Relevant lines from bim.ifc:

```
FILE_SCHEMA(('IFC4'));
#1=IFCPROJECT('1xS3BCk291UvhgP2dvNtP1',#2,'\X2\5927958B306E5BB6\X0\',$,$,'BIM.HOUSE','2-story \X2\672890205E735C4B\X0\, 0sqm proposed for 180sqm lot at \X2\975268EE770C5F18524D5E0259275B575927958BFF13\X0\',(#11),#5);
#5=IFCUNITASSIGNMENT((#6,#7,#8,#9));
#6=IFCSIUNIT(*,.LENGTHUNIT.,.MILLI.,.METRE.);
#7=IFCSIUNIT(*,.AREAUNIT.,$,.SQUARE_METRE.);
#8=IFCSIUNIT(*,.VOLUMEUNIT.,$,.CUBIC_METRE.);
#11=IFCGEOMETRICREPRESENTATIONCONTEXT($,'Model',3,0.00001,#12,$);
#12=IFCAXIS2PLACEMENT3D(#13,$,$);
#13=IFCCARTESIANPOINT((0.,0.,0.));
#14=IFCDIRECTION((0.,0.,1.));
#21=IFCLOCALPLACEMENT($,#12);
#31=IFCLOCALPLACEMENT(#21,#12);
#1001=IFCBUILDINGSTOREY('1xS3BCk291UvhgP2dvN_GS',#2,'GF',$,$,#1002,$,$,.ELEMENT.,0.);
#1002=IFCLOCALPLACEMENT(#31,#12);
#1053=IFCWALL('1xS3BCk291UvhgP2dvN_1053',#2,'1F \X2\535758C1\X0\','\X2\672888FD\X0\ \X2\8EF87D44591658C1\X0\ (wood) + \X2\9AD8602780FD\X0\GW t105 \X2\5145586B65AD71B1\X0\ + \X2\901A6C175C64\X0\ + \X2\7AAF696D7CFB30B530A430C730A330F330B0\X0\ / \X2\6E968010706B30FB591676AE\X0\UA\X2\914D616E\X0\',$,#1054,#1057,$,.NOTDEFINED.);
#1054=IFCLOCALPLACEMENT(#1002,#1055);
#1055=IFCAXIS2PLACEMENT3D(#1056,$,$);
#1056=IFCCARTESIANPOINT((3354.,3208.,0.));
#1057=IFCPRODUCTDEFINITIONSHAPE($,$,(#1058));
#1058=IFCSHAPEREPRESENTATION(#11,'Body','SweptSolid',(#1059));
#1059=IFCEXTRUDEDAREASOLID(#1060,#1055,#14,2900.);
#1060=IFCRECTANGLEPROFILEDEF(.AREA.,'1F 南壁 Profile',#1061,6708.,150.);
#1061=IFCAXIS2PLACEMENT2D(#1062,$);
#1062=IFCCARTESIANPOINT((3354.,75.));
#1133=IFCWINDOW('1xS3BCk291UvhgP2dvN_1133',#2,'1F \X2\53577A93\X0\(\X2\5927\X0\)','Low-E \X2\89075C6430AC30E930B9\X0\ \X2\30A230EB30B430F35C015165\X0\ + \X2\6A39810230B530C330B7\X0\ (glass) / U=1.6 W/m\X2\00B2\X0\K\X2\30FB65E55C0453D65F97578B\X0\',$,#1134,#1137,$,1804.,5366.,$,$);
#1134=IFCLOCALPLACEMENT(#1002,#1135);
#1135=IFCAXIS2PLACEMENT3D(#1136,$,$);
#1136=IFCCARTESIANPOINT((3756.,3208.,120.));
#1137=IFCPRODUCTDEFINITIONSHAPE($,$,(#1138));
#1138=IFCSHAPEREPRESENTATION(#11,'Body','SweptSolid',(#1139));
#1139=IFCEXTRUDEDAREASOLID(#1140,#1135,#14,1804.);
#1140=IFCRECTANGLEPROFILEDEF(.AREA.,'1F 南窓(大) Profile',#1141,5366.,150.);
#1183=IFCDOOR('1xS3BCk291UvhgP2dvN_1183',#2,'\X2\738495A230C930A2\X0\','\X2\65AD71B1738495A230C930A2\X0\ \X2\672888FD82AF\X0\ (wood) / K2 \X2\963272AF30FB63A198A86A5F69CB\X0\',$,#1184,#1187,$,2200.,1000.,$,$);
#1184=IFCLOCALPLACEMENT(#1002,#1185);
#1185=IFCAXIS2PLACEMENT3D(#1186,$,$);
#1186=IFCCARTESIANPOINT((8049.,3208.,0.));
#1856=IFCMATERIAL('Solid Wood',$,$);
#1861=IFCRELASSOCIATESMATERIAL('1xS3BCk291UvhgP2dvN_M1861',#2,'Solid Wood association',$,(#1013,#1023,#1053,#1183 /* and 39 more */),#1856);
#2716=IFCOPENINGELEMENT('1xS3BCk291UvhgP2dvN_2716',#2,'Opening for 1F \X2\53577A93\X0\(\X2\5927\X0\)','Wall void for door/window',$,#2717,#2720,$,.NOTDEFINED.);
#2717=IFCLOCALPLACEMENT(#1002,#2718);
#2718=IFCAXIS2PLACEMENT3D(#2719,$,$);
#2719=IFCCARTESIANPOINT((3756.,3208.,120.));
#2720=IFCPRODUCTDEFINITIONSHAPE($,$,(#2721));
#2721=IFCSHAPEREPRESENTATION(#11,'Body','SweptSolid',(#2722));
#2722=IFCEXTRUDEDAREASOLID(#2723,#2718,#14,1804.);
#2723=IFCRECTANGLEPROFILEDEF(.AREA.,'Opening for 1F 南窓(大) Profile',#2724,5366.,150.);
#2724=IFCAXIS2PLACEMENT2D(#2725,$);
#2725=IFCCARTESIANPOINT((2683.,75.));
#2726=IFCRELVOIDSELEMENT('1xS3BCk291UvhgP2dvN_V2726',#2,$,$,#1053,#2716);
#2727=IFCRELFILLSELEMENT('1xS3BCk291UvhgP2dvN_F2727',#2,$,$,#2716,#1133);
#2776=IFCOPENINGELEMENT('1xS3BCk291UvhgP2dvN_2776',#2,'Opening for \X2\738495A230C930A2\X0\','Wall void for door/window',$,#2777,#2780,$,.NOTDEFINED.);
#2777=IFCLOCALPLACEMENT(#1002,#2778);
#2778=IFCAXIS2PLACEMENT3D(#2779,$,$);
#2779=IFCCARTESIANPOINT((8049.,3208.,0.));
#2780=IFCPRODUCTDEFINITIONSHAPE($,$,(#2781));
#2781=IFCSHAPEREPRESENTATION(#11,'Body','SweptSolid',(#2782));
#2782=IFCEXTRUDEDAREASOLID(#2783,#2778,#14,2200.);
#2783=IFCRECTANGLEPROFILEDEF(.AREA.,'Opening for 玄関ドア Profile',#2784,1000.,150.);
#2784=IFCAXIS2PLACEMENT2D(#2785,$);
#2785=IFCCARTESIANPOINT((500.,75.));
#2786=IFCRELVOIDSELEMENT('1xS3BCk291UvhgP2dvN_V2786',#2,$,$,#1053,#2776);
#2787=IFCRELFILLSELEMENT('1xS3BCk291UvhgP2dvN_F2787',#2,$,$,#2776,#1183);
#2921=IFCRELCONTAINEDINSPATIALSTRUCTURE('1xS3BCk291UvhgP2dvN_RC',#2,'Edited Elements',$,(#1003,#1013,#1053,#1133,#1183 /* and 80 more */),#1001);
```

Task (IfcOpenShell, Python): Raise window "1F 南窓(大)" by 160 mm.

```python
import numpy as np
import ifcopenshell
import ifcopenshell.api.geometry
import ifcopenshell.util.placement
import ifcopenshell.util.unit

model = ifcopenshell.open("bim.ifc")
unit_scale = ifcopenshell.util.unit.calculate_unit_scale(model)

window = model.by_id(1133)
opening = window.FillsVoids[0].RelatingOpeningElement
dz = 160.0

shift = np.array([0.0, 0.0, dz])
# The window is not placed relative to its opening, so move both.
for product in (opening, window):
    matrix = ifcopenshell.util.placement.get_local_placement(product.ObjectPlacement)
    matrix[:3, 3] += shift
    ifcopenshell.api.geometry.edit_object_placement(model, product=product, matrix=matrix, is_si=False)

print(f"moved by {dz * unit_scale:+.3f} m")

model.write("bim-out.ifc")
```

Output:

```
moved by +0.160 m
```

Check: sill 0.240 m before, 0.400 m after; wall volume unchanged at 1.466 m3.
